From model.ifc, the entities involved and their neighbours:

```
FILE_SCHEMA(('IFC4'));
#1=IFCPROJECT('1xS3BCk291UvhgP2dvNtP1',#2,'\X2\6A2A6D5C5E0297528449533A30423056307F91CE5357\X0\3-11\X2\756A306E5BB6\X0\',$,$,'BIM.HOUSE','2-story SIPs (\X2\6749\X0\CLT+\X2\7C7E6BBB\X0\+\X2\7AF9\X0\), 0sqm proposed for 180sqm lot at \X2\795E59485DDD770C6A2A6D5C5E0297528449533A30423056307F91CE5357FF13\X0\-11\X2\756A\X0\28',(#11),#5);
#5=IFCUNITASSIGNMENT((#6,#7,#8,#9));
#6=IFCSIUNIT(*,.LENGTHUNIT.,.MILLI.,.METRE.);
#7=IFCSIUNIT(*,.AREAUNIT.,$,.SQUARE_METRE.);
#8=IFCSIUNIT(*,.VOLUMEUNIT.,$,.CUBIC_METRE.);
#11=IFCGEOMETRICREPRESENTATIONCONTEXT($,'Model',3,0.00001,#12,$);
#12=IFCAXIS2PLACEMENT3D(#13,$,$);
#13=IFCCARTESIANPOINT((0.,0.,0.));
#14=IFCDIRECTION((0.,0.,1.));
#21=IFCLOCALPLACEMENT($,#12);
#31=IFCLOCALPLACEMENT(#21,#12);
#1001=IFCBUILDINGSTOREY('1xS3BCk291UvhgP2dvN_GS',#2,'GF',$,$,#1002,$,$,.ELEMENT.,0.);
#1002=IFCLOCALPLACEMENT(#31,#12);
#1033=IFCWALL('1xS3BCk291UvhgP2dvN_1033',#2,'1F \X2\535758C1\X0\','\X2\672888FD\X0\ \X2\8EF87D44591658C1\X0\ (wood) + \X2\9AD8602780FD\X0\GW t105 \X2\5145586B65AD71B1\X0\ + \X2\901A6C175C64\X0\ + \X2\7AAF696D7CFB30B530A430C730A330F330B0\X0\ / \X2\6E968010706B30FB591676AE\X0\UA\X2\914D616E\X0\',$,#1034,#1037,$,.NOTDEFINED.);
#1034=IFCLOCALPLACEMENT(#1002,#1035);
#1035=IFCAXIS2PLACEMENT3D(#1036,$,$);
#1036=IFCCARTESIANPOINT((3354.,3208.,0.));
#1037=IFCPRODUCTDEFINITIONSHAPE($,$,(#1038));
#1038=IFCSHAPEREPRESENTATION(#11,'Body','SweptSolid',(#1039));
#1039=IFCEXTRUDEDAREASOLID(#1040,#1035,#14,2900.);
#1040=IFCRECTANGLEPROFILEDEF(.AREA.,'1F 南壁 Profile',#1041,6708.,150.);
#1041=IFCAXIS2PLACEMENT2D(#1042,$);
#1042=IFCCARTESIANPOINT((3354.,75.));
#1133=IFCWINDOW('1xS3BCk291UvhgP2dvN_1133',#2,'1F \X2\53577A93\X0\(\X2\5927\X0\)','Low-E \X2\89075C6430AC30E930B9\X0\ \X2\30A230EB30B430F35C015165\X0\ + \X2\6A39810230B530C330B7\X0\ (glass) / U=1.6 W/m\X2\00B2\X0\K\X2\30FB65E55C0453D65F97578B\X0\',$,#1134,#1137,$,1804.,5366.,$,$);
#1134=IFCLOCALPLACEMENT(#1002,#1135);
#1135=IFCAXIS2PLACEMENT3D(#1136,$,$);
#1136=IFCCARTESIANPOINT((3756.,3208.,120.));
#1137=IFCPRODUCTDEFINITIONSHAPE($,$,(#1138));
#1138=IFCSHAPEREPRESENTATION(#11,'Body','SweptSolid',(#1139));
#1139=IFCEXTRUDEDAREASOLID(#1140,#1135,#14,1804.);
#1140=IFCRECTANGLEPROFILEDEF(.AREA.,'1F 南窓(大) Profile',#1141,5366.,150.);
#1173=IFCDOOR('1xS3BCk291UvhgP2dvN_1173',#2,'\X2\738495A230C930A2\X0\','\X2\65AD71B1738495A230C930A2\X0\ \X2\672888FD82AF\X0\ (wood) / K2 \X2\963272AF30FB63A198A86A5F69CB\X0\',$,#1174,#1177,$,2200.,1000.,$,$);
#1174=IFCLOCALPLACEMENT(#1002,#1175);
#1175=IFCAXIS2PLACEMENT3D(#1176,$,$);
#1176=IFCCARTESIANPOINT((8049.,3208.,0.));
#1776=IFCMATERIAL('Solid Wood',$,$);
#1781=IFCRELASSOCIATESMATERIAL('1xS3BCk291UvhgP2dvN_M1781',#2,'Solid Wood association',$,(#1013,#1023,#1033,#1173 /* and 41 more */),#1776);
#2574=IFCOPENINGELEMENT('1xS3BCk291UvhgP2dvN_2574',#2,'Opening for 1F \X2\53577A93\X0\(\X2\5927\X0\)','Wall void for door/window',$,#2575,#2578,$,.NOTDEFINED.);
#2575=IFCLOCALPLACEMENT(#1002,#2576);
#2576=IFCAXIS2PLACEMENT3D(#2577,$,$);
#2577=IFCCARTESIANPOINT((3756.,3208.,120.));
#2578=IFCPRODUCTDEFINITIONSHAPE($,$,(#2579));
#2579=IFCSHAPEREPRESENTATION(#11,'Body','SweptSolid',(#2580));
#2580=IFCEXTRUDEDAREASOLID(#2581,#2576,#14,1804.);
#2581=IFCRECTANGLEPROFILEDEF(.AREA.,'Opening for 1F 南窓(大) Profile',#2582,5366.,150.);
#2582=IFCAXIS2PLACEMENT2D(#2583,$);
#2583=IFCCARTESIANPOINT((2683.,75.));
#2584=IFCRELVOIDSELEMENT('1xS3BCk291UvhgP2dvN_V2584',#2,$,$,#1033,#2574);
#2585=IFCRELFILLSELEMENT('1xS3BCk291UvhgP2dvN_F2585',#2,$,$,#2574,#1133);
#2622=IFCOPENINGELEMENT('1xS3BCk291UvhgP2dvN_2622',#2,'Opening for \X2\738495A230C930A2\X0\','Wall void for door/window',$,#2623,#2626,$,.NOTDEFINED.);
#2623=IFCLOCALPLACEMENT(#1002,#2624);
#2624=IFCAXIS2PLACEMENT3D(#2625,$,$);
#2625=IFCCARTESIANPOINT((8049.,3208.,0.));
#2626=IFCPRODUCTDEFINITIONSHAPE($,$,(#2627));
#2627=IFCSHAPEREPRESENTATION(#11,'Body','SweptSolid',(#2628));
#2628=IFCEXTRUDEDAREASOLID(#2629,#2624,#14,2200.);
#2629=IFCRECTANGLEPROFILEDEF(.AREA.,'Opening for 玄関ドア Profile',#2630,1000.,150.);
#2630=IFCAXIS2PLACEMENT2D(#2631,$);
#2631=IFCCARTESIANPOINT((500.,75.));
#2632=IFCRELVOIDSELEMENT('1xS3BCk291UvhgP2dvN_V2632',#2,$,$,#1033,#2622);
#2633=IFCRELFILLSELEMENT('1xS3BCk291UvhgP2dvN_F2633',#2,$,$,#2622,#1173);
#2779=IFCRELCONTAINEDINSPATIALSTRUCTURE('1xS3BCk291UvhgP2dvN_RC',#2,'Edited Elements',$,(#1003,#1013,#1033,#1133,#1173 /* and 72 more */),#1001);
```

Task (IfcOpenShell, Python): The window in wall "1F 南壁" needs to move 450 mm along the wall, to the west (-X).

```python
import ifcopenshell
import ifcopenshell.api.geometry
import ifcopenshell.util.placement

model = ifcopenshell.open("model.ifc")

window = model.by_guid("1xS3BCk291UvhgP2dvN_1133")
opening = window.FillsVoids[0].RelatingOpeningElement
wall = opening.VoidsElements[0].RelatingBuildingElement

wall_matrix = ifcopenshell.util.placement.get_local_placement(wall.ObjectPlacement)
shift = wall_matrix[:3, 0] * -450.0
before = ifcopenshell.util.placement.get_local_placement(window.ObjectPlacement)[:3, 3].copy()

# The window is not placed relative to its opening, so move both.
for product in (opening, window):
    matrix = ifcopenshell.util.placement.get_local_placement(product.ObjectPlacement)
    matrix[:3, 3] += shift
    ifcopenshell.api.geometry.edit_object_placement(model, product=product, matrix=matrix, is_si=False)

after = ifcopenshell.util.placement.get_local_placement(window.ObjectPlacement)[:3, 3]
print("window moved by", (after - before).round(3) + 0.0)

model.write("model-out.ifc")
```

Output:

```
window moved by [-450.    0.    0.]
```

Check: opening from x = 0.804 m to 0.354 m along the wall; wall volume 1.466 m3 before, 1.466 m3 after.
